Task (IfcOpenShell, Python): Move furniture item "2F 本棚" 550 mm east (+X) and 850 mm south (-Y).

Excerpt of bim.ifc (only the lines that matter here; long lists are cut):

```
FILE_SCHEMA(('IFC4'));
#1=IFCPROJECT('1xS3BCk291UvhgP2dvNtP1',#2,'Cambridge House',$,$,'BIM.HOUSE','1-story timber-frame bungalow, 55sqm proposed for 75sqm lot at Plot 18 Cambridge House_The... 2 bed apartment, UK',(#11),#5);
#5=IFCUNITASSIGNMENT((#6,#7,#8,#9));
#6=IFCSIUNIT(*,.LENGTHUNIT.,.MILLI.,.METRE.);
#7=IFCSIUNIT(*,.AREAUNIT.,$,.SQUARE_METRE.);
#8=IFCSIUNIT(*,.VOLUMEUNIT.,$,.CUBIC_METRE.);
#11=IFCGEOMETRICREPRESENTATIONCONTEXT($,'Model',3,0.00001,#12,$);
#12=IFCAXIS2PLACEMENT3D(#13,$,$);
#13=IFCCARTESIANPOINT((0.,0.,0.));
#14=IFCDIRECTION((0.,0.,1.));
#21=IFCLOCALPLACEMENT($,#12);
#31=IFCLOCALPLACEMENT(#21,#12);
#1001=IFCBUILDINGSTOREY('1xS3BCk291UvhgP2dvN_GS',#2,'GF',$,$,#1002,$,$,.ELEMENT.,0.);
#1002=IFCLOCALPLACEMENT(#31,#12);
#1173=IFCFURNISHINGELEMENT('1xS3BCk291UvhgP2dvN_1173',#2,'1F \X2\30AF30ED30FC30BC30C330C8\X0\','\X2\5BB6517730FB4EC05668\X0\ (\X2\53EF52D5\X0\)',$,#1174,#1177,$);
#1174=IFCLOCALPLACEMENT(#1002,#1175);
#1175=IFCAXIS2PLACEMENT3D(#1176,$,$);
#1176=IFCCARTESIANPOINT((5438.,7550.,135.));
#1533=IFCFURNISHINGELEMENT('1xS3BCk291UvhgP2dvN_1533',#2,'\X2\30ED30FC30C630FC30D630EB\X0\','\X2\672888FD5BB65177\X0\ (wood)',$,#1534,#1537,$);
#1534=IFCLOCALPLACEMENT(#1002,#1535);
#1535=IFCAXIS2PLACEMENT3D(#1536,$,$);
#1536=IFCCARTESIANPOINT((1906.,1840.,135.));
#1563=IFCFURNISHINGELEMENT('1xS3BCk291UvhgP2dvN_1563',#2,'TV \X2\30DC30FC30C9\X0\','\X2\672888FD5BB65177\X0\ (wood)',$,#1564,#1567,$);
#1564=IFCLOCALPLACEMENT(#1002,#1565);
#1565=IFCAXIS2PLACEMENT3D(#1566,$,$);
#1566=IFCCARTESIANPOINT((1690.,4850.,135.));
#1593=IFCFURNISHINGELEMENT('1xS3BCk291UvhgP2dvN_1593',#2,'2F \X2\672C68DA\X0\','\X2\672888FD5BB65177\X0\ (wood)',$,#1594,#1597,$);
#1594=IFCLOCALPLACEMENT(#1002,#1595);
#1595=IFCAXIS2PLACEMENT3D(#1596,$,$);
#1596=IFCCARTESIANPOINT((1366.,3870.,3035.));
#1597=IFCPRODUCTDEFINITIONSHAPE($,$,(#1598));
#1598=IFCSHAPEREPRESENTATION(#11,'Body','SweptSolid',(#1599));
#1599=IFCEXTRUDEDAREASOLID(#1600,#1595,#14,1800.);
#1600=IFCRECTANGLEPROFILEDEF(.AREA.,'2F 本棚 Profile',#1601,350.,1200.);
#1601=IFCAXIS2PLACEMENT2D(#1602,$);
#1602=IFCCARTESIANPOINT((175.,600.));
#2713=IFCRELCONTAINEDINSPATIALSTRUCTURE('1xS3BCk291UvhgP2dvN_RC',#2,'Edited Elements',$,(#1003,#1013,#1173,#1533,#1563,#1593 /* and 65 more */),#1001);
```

```python
import ifcopenshell
import ifcopenshell.api.geometry
import ifcopenshell.util.placement
import ifcopenshell.util.unit

model = ifcopenshell.open("bim.ifc")
unit_scale = ifcopenshell.util.unit.calculate_unit_scale(model)

item = model.by_guid("1xS3BCk291UvhgP2dvN_1593")
matrix = ifcopenshell.util.placement.get_local_placement(item.ObjectPlacement)
matrix[0, 3] += 0.55 / unit_scale
matrix[1, 3] -= 0.85 / unit_scale
ifcopenshell.api.geometry.edit_object_placement(model, product=item, matrix=matrix, is_si=False)

print(ifcopenshell.util.placement.get_local_placement(item.ObjectPlacement).round(3) + 0.0)

model.write("bim_v2.ifc")
```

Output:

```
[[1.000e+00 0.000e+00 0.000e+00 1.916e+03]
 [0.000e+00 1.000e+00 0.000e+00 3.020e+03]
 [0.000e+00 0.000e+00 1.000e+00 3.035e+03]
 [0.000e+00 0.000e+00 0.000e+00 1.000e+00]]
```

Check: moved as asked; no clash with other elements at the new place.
